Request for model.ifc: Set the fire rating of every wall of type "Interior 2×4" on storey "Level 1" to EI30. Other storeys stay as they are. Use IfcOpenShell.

First a look at what the model holds.

```python
import ifcopenshell
import ifcopenshell.util.element

model = ifcopenshell.open("model.ifc")
print(model.schema)
storey = next(s for s in model.by_type("IfcBuildingStorey") if s.Name == "Level 1")
walls = [e for e in ifcopenshell.util.element.get_decomposition(storey) if e.is_a("IfcWall")]
seen = {}
for e in walls:
    element_type = ifcopenshell.util.element.get_type(e)
    key = (element_type.Name if element_type != e and element_type else None, ifcopenshell.util.element.get_pset(e, "Pset_WallCommon", "FireRating"))
    seen[key] = seen.get(key, 0) + 1
for (name, value), count in sorted(seen.items(), key=str):
    print(count, "x", name, "|", value)
```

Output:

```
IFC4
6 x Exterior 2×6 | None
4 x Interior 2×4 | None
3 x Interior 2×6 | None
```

```python
import ifcopenshell
import ifcopenshell.api.pset
import ifcopenshell.util.element

model = ifcopenshell.open("model.ifc")

storey = next(s for s in model.by_type("IfcBuildingStorey") if s.Name == "Level 1")
walls = [e for e in ifcopenshell.util.element.get_decomposition(storey) if e.is_a("IfcWall")]

count = 0
for e in walls:
    element_type = ifcopenshell.util.element.get_type(e)
    if element_type in (None, e) or element_type.Name != "Interior 2×4":
        continue
    # add_pset returns the element's existing set when there is one.
    pset = ifcopenshell.api.pset.add_pset(model, product=e, name="Pset_WallCommon")
    ifcopenshell.api.pset.edit_pset(model, pset=pset, properties={"FireRating": "EI30"})
    count += 1

print(count, "walls updated")

model.write("model-out.ifc")
```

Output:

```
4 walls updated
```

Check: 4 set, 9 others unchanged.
